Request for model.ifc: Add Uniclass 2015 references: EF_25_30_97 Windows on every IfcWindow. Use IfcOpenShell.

First a look at what the model holds.

```python
import ifcopenshell

model = ifcopenshell.open("model.ifc")
print(model.schema)
print("classifications:", [c.Name for c in model.by_type("IfcClassification")])
for ifc_class in ("IfcDoor", "IfcRoof", "IfcStair", "IfcWall", "IfcWindow"):
    print(ifc_class, len(model.by_type(ifc_class)))
```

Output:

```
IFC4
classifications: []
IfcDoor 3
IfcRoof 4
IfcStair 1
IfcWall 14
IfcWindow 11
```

```python
import ifcopenshell
import ifcopenshell.api.classification

model = ifcopenshell.open("model.ifc")

system = ifcopenshell.api.classification.add_classification(model, classification="Uniclass 2015")

codes = {
    "IfcWindow": ("EF_25_30_97", "Windows"),
}
for ifc_class, (code, name) in codes.items():
    products = model.by_type(ifc_class)
    ifcopenshell.api.classification.add_reference(
        model, products=products, classification=system, identification=code, name=name
    )
    print(code, len(products))

model.write("model_rev.ifc")
```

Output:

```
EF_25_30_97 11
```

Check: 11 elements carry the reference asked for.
